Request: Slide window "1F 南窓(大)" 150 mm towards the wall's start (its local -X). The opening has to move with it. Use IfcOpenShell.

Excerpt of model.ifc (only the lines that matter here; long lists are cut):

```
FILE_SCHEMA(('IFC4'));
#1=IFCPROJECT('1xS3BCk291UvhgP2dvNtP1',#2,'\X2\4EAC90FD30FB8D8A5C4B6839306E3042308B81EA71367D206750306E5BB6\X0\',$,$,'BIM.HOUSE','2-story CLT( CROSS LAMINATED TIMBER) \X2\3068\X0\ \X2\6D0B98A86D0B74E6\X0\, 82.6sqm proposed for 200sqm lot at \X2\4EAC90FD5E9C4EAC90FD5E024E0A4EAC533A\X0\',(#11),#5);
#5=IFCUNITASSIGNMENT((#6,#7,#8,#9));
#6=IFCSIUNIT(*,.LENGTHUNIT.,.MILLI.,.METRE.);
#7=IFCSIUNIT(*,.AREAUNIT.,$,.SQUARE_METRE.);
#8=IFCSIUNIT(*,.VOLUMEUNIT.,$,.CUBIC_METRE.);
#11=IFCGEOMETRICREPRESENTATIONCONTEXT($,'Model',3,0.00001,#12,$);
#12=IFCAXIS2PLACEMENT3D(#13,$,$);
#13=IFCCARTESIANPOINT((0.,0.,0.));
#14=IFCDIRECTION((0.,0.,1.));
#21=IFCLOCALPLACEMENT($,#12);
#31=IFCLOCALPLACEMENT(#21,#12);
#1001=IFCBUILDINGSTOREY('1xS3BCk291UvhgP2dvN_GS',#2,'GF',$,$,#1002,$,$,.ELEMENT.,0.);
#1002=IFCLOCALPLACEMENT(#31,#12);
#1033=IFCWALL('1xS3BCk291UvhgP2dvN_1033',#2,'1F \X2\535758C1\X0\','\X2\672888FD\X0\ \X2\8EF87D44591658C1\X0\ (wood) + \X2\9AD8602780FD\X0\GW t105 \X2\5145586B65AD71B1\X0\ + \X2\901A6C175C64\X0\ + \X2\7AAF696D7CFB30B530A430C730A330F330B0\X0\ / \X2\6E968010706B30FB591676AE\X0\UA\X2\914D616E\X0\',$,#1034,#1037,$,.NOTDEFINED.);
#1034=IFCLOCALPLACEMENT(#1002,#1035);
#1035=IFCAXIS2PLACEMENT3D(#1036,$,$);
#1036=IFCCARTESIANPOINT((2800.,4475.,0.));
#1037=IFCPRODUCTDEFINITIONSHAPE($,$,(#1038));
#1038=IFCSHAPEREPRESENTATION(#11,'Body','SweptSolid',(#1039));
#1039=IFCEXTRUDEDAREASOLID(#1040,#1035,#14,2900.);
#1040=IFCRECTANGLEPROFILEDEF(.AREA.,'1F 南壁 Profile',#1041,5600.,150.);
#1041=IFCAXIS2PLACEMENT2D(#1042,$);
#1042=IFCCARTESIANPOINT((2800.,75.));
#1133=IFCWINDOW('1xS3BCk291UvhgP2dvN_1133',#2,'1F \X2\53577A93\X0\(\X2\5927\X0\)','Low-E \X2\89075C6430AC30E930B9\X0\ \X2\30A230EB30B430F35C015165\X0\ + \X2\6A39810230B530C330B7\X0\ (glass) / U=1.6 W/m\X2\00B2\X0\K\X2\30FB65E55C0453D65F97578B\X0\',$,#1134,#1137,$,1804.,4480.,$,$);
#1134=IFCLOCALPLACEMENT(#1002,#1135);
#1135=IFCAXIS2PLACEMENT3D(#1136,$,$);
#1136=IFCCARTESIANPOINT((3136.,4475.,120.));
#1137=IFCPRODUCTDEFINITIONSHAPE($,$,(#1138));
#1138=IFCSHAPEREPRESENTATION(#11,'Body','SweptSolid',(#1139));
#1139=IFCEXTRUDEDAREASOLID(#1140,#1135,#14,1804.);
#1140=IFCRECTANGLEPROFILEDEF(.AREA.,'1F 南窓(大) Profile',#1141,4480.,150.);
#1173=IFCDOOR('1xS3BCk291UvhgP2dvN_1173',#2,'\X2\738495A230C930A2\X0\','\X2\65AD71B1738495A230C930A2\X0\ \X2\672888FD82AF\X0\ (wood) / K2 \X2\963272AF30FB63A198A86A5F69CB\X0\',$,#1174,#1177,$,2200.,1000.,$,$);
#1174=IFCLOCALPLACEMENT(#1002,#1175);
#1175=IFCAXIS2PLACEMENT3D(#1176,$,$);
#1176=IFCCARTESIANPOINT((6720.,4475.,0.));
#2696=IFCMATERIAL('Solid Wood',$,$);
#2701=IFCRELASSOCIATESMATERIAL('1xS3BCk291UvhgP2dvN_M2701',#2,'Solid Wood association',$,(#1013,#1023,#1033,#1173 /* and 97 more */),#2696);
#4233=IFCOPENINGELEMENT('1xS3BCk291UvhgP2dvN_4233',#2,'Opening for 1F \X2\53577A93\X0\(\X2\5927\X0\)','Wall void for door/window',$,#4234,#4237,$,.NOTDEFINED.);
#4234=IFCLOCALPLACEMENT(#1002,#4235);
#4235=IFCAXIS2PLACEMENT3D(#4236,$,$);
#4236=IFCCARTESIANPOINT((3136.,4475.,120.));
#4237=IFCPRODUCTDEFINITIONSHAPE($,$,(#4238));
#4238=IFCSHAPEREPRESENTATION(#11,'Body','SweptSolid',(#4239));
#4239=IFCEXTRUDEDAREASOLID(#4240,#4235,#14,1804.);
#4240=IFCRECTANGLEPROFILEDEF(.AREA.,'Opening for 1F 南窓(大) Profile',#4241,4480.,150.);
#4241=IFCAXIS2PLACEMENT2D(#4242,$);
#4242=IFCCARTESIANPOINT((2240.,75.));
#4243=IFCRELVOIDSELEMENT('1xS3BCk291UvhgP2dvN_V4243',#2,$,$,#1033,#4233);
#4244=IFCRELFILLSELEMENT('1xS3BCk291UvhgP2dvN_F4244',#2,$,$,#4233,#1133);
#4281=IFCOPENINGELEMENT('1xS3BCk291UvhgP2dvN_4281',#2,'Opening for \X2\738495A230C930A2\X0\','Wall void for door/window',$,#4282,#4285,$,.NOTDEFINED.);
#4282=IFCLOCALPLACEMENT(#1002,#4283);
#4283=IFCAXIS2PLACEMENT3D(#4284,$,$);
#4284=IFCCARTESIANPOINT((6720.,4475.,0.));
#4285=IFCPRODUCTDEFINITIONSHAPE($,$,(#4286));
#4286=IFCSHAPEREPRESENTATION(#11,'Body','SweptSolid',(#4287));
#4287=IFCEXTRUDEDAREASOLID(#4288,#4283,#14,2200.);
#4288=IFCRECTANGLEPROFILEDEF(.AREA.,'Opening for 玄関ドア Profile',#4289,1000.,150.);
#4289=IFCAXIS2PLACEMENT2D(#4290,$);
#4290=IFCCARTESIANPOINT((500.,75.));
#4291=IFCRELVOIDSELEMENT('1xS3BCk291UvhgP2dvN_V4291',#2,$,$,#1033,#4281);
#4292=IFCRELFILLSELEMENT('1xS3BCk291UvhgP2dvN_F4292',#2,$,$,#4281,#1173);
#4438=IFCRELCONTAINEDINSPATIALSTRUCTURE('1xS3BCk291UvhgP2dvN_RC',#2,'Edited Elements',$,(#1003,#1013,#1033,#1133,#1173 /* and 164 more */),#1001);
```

```python
import ifcopenshell
import ifcopenshell.api.geometry
import ifcopenshell.util.placement

model = ifcopenshell.open("model.ifc")

window = model.by_id(1133)
opening = window.FillsVoids[0].RelatingOpeningElement
wall = opening.VoidsElements[0].RelatingBuildingElement

wall_matrix = ifcopenshell.util.placement.get_local_placement(wall.ObjectPlacement)
shift = wall_matrix[:3, 0] * -150.0
before = ifcopenshell.util.placement.get_local_placement(window.ObjectPlacement)[:3, 3].copy()

# The window is not placed relative to its opening, so move both.
for product in (opening, window):
    matrix = ifcopenshell.util.placement.get_local_placement(product.ObjectPlacement)
    matrix[:3, 3] += shift
    ifcopenshell.api.geometry.edit_object_placement(model, product=product, matrix=matrix, is_si=False)

after = ifcopenshell.util.placement.get_local_placement(window.ObjectPlacement)[:3, 3]
print("window moved by", (after - before).round(3) + 0.0)

model.write("model_v2.ifc")
```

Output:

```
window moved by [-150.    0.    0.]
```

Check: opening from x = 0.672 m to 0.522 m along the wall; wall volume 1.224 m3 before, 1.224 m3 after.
